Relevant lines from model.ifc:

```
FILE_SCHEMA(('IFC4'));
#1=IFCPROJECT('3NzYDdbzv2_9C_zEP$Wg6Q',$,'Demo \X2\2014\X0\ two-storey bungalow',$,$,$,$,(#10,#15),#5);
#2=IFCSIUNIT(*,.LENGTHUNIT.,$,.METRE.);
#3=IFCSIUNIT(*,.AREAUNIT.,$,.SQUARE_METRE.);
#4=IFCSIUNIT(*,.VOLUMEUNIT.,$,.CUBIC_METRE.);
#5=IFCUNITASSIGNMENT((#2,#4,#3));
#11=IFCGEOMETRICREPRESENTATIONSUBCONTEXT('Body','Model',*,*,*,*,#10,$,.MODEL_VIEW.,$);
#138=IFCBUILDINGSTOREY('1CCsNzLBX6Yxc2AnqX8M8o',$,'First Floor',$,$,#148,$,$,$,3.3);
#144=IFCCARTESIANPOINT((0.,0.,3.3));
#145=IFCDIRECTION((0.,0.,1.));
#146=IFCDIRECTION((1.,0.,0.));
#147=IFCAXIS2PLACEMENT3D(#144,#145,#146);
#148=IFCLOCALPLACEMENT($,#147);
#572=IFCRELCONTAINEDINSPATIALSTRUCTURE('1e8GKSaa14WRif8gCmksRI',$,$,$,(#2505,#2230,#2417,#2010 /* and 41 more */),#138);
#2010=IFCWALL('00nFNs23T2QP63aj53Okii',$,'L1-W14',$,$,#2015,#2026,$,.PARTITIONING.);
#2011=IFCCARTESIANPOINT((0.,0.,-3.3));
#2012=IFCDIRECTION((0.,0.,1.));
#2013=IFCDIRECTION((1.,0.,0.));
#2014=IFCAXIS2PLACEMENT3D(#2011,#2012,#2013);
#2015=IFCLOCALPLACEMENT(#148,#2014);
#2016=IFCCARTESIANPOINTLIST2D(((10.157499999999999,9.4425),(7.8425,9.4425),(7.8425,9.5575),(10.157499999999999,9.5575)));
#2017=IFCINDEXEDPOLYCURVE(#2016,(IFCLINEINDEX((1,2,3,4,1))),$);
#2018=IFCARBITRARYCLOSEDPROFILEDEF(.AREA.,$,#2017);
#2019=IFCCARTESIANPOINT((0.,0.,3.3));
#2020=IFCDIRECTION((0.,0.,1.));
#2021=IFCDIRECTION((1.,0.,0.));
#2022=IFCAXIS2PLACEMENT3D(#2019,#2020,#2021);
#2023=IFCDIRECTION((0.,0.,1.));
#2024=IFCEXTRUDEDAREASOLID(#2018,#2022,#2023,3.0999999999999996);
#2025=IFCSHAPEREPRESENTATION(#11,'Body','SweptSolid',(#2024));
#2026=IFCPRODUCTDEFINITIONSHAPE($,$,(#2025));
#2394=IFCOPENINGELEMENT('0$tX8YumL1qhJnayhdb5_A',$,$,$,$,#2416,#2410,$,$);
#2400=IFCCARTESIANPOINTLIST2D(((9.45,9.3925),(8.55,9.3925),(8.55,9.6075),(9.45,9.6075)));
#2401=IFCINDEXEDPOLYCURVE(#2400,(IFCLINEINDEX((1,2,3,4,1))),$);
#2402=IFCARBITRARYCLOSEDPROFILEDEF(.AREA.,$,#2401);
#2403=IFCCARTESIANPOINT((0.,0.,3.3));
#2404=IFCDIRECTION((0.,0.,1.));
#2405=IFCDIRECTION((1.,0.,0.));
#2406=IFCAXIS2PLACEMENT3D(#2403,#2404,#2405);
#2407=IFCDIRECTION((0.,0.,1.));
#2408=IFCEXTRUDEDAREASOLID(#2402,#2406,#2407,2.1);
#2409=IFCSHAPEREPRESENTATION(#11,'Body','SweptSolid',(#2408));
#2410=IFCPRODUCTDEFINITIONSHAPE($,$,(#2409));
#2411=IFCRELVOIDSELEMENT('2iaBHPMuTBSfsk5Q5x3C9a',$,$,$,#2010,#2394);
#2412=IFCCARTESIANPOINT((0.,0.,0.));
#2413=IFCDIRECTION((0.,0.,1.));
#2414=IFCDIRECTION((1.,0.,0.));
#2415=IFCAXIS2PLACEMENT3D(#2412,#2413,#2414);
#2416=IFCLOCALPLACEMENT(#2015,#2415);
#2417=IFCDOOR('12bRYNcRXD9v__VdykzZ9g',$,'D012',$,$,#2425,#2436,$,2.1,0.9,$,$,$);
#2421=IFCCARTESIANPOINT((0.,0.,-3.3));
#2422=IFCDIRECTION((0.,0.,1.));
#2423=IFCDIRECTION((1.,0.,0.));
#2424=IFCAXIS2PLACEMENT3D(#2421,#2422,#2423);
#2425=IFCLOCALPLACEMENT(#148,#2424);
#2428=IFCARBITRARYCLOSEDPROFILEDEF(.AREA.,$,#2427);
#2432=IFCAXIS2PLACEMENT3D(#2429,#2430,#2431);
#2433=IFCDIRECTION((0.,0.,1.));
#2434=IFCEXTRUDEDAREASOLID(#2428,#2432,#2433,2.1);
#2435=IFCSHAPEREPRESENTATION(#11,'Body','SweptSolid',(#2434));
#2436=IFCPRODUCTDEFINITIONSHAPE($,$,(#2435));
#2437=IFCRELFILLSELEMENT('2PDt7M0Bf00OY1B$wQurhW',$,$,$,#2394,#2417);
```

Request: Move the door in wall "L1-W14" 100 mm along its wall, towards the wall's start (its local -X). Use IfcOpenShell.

```python
import ifcopenshell
import ifcopenshell.api.geometry
import ifcopenshell.util.placement
import ifcopenshell.util.unit

model = ifcopenshell.open("model.ifc")
unit_scale = ifcopenshell.util.unit.calculate_unit_scale(model)

door = model.by_id(2417)
opening = door.FillsVoids[0].RelatingOpeningElement
wall = opening.VoidsElements[0].RelatingBuildingElement

wall_matrix = ifcopenshell.util.placement.get_local_placement(wall.ObjectPlacement)
shift = wall_matrix[:3, 0] * -0.1 / unit_scale
before = ifcopenshell.util.placement.get_local_placement(door.ObjectPlacement)[:3, 3].copy()

# The door is not placed relative to its opening, so move both.
for product in (opening, door):
    matrix = ifcopenshell.util.placement.get_local_placement(product.ObjectPlacement)
    matrix[:3, 3] += shift
    ifcopenshell.api.geometry.edit_object_placement(model, product=product, matrix=matrix, is_si=False)

after = ifcopenshell.util.placement.get_local_placement(door.ObjectPlacement)[:3, 3]
print("door moved by", (after - before).round(3) + 0.0)

model.write("model-out.ifc")
```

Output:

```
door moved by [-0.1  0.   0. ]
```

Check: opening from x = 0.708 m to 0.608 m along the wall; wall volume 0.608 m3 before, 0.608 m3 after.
